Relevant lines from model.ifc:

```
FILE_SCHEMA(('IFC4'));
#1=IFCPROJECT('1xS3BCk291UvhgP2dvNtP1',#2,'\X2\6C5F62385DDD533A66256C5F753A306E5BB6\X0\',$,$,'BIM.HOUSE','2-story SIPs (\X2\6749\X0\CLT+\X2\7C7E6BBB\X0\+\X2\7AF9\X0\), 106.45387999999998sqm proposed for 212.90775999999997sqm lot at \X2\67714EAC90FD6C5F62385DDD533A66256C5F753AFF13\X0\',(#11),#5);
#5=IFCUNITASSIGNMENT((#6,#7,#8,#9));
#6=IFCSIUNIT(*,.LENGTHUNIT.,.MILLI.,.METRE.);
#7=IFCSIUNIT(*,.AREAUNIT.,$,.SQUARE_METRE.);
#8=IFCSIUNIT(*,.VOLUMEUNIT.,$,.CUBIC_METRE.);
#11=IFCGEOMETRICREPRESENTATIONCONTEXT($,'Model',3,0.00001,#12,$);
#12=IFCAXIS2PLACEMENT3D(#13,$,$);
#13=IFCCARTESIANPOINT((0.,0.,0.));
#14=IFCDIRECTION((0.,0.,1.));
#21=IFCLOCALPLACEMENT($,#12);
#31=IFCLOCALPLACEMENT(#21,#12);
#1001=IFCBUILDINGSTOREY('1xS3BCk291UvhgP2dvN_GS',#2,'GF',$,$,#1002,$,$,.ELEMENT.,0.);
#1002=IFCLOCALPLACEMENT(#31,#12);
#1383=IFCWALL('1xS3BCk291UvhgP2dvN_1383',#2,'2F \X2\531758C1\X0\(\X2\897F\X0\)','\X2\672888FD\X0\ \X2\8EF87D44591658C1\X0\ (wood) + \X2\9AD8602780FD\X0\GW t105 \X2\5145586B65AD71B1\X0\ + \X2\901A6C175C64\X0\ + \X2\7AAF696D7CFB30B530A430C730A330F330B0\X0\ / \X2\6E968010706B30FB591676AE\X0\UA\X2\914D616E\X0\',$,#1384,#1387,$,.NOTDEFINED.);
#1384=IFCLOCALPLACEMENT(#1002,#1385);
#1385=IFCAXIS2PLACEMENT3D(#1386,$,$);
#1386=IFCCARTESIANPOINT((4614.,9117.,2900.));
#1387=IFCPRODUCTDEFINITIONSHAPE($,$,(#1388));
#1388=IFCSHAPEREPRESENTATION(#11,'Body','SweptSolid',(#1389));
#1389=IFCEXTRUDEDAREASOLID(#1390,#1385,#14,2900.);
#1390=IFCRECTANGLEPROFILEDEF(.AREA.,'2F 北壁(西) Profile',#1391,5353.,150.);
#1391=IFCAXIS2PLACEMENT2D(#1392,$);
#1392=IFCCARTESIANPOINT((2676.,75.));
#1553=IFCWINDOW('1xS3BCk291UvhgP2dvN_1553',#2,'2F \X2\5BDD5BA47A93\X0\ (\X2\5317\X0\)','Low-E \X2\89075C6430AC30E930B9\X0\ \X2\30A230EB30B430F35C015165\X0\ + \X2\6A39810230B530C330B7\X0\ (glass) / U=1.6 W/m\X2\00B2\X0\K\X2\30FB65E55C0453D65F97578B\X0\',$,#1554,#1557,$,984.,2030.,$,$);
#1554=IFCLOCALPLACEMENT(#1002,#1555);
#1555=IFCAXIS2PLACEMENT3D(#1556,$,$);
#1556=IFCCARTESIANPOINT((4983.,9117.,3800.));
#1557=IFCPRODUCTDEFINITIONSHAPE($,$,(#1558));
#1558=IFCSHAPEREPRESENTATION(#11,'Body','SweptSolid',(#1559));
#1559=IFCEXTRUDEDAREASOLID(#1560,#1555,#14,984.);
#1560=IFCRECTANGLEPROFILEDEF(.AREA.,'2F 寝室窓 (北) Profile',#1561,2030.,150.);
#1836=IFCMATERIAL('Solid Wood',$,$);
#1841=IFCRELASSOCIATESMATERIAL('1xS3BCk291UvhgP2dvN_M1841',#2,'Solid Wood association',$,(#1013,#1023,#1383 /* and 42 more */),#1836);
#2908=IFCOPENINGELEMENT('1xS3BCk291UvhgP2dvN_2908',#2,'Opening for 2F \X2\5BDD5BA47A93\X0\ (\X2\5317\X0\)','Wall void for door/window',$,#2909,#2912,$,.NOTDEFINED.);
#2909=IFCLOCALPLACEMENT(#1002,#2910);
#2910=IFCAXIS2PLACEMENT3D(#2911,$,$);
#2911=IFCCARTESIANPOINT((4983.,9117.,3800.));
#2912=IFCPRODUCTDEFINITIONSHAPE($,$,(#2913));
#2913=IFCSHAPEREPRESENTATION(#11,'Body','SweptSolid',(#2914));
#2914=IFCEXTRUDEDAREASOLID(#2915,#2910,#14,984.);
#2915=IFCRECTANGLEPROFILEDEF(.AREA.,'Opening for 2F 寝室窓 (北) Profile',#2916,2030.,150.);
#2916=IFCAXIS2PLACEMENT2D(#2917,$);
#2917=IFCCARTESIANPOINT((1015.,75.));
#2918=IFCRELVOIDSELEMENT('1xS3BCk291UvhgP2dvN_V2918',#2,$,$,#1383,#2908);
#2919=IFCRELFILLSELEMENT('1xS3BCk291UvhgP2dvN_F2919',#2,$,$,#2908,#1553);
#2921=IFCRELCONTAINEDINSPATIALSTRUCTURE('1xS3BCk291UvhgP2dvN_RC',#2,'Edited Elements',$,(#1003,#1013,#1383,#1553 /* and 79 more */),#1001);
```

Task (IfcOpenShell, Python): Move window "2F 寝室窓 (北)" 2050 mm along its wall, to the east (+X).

```python
import ifcopenshell
import ifcopenshell.api.geometry
import ifcopenshell.util.placement
import ifcopenshell.util.unit

model = ifcopenshell.open("model.ifc")
unit_scale = ifcopenshell.util.unit.calculate_unit_scale(model)

window = model.by_id(1553)
opening = window.FillsVoids[0].RelatingOpeningElement
wall = opening.VoidsElements[0].RelatingBuildingElement

wall_matrix = ifcopenshell.util.placement.get_local_placement(wall.ObjectPlacement)
shift = wall_matrix[:3, 0] * 2.05 / unit_scale
before = ifcopenshell.util.placement.get_local_placement(window.ObjectPlacement)[:3, 3].copy()

# The window is not placed relative to its opening, so move both.
for product in (opening, window):
    matrix = ifcopenshell.util.placement.get_local_placement(product.ObjectPlacement)
    matrix[:3, 3] += shift
    ifcopenshell.api.geometry.edit_object_placement(model, product=product, matrix=matrix, is_si=False)

after = ifcopenshell.util.placement.get_local_placement(window.ObjectPlacement)[:3, 3]
print("window moved by", (after - before).round(3) + 0.0)

model.write("model_updated.ifc")
```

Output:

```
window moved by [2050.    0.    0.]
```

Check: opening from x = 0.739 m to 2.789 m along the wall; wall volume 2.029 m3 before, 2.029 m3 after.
